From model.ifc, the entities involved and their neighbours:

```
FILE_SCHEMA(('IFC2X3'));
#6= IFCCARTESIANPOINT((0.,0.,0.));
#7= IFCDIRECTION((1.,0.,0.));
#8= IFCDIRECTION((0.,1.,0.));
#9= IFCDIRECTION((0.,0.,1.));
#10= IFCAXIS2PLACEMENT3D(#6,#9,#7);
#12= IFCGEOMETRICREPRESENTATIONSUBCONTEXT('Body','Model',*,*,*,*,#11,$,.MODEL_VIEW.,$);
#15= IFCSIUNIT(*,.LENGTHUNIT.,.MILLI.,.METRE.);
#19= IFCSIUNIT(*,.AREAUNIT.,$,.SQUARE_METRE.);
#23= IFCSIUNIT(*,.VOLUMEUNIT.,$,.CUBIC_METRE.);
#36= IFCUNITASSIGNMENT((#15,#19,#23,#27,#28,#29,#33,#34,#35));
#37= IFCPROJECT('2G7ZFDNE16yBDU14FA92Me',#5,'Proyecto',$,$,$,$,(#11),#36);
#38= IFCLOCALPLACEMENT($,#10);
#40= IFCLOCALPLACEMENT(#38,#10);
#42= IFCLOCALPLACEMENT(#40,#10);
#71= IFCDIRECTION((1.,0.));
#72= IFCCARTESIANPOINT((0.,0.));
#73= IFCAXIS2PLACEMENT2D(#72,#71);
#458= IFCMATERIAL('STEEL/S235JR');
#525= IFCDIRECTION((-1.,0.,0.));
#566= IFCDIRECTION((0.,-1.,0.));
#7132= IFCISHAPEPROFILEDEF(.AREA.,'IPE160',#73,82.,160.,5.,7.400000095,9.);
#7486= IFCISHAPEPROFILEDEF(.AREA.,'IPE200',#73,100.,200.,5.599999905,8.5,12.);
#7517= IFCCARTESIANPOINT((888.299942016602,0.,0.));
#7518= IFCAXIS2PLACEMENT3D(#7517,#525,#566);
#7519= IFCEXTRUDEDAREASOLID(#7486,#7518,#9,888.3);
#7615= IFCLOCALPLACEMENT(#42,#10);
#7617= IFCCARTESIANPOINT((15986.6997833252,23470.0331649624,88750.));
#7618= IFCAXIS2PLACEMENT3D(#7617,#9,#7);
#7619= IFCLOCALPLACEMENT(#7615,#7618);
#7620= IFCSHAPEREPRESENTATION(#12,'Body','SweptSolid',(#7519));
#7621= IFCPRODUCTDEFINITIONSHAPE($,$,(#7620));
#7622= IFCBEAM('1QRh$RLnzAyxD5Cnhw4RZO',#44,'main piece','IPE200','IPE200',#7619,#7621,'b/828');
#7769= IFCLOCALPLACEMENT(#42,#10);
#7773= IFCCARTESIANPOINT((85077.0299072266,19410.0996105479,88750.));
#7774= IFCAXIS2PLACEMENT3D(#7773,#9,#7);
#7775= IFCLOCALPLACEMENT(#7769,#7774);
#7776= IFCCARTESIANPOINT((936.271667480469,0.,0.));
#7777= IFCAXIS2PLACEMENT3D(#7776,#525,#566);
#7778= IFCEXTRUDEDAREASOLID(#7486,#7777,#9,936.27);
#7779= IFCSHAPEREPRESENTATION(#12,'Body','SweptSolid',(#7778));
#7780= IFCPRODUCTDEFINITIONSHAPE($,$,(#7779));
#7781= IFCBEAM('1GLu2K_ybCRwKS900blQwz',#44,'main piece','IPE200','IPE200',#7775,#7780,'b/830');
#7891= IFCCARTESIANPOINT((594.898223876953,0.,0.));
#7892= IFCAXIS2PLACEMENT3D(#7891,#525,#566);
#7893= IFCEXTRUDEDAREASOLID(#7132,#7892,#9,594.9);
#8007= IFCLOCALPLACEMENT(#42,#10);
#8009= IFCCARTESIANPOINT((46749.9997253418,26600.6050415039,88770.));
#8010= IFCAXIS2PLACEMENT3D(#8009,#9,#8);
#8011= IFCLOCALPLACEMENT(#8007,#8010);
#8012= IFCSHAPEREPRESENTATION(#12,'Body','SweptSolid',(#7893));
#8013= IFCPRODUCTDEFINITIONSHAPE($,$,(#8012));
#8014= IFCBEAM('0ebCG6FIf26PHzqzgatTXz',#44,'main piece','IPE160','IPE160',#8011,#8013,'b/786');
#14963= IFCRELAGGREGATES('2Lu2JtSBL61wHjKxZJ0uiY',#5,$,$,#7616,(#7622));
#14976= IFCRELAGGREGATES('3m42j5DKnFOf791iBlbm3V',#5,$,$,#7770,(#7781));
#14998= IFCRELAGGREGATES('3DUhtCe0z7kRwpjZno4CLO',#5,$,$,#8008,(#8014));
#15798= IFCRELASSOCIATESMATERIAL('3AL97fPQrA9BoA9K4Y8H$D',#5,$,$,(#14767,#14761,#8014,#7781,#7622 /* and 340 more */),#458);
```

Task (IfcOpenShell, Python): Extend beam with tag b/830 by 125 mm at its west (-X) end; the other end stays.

```python
import ifcopenshell
import ifcopenshell.util.representation
import ifcopenshell.util.unit

model = ifcopenshell.open("model.ifc")
unit_scale = ifcopenshell.util.unit.calculate_unit_scale(model)

member = model.by_guid("1GLu2K_ybCRwKS900blQwz")
change = 0.125 / unit_scale

# The extrusion runs towards the end named, so only its depth changes.
body = ifcopenshell.util.representation.get_representation(member, "Model", "Body")
solid = body.Items[0]
old_length = solid.Depth
solid.Depth += change

print(f"length {old_length:g} -> {solid.Depth:g}")

model.write("model_rev.ifc")
```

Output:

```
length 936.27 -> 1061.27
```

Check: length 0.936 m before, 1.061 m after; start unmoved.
